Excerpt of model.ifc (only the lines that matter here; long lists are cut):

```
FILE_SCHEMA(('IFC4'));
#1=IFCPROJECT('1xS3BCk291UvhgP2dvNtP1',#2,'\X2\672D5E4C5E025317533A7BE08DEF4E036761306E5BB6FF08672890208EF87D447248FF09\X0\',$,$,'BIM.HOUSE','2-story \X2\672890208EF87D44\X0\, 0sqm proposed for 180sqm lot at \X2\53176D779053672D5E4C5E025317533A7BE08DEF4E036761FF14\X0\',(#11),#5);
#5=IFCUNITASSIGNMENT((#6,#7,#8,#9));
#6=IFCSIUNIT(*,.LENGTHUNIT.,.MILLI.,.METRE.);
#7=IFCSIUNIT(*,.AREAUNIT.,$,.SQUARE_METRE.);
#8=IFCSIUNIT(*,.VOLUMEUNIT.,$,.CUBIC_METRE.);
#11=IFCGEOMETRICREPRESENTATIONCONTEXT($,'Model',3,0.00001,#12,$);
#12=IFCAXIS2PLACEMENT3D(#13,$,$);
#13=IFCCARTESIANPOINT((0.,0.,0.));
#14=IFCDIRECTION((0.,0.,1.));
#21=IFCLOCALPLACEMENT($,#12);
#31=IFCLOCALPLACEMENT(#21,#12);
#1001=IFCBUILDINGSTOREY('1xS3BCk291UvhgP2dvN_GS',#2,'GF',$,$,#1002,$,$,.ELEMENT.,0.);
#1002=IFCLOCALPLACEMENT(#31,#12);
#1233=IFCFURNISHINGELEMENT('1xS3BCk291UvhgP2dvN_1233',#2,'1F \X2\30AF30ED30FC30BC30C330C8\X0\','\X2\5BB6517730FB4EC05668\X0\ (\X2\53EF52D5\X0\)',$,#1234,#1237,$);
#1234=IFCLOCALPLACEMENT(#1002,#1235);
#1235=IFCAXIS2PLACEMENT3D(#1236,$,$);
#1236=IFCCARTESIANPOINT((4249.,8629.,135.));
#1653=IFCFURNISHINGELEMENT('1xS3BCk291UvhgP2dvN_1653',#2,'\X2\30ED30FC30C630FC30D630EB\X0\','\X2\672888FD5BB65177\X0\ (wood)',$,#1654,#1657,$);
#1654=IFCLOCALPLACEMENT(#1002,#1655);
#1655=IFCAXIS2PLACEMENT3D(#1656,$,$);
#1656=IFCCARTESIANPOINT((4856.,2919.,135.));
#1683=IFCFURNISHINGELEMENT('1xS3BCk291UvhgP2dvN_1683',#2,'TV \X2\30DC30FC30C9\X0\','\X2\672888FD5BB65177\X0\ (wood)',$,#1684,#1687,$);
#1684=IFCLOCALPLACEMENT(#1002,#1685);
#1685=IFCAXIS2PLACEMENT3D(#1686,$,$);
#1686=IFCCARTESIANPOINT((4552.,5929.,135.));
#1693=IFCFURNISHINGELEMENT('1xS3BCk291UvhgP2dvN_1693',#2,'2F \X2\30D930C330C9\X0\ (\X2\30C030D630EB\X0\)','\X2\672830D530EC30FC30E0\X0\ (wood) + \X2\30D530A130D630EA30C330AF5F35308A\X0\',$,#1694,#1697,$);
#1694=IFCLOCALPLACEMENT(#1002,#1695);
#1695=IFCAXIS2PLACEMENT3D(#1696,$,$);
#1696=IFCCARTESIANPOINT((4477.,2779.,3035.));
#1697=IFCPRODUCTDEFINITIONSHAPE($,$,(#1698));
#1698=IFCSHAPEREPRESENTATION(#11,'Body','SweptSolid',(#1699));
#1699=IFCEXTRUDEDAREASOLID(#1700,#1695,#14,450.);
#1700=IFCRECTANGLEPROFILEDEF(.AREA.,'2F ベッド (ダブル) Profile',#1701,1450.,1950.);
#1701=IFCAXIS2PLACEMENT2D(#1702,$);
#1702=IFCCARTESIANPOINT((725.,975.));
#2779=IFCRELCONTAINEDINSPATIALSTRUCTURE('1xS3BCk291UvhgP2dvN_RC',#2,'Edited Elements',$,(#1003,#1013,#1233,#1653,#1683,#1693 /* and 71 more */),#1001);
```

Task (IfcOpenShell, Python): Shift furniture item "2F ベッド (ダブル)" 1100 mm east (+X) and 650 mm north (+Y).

```python
import ifcopenshell
import ifcopenshell.api.geometry
import ifcopenshell.util.placement

model = ifcopenshell.open("model.ifc")

item = model.by_id(1693)
matrix = ifcopenshell.util.placement.get_local_placement(item.ObjectPlacement)
matrix[0, 3] += 1100.0
matrix[1, 3] += 650.0
ifcopenshell.api.geometry.edit_object_placement(model, product=item, matrix=matrix, is_si=False)

print(ifcopenshell.util.placement.get_local_placement(item.ObjectPlacement).round(3) + 0.0)

model.write("model-out.ifc")
```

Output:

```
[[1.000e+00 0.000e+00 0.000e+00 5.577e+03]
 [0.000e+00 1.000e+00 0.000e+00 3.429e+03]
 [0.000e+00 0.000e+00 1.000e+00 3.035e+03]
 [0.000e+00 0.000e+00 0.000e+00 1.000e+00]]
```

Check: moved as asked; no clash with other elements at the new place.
